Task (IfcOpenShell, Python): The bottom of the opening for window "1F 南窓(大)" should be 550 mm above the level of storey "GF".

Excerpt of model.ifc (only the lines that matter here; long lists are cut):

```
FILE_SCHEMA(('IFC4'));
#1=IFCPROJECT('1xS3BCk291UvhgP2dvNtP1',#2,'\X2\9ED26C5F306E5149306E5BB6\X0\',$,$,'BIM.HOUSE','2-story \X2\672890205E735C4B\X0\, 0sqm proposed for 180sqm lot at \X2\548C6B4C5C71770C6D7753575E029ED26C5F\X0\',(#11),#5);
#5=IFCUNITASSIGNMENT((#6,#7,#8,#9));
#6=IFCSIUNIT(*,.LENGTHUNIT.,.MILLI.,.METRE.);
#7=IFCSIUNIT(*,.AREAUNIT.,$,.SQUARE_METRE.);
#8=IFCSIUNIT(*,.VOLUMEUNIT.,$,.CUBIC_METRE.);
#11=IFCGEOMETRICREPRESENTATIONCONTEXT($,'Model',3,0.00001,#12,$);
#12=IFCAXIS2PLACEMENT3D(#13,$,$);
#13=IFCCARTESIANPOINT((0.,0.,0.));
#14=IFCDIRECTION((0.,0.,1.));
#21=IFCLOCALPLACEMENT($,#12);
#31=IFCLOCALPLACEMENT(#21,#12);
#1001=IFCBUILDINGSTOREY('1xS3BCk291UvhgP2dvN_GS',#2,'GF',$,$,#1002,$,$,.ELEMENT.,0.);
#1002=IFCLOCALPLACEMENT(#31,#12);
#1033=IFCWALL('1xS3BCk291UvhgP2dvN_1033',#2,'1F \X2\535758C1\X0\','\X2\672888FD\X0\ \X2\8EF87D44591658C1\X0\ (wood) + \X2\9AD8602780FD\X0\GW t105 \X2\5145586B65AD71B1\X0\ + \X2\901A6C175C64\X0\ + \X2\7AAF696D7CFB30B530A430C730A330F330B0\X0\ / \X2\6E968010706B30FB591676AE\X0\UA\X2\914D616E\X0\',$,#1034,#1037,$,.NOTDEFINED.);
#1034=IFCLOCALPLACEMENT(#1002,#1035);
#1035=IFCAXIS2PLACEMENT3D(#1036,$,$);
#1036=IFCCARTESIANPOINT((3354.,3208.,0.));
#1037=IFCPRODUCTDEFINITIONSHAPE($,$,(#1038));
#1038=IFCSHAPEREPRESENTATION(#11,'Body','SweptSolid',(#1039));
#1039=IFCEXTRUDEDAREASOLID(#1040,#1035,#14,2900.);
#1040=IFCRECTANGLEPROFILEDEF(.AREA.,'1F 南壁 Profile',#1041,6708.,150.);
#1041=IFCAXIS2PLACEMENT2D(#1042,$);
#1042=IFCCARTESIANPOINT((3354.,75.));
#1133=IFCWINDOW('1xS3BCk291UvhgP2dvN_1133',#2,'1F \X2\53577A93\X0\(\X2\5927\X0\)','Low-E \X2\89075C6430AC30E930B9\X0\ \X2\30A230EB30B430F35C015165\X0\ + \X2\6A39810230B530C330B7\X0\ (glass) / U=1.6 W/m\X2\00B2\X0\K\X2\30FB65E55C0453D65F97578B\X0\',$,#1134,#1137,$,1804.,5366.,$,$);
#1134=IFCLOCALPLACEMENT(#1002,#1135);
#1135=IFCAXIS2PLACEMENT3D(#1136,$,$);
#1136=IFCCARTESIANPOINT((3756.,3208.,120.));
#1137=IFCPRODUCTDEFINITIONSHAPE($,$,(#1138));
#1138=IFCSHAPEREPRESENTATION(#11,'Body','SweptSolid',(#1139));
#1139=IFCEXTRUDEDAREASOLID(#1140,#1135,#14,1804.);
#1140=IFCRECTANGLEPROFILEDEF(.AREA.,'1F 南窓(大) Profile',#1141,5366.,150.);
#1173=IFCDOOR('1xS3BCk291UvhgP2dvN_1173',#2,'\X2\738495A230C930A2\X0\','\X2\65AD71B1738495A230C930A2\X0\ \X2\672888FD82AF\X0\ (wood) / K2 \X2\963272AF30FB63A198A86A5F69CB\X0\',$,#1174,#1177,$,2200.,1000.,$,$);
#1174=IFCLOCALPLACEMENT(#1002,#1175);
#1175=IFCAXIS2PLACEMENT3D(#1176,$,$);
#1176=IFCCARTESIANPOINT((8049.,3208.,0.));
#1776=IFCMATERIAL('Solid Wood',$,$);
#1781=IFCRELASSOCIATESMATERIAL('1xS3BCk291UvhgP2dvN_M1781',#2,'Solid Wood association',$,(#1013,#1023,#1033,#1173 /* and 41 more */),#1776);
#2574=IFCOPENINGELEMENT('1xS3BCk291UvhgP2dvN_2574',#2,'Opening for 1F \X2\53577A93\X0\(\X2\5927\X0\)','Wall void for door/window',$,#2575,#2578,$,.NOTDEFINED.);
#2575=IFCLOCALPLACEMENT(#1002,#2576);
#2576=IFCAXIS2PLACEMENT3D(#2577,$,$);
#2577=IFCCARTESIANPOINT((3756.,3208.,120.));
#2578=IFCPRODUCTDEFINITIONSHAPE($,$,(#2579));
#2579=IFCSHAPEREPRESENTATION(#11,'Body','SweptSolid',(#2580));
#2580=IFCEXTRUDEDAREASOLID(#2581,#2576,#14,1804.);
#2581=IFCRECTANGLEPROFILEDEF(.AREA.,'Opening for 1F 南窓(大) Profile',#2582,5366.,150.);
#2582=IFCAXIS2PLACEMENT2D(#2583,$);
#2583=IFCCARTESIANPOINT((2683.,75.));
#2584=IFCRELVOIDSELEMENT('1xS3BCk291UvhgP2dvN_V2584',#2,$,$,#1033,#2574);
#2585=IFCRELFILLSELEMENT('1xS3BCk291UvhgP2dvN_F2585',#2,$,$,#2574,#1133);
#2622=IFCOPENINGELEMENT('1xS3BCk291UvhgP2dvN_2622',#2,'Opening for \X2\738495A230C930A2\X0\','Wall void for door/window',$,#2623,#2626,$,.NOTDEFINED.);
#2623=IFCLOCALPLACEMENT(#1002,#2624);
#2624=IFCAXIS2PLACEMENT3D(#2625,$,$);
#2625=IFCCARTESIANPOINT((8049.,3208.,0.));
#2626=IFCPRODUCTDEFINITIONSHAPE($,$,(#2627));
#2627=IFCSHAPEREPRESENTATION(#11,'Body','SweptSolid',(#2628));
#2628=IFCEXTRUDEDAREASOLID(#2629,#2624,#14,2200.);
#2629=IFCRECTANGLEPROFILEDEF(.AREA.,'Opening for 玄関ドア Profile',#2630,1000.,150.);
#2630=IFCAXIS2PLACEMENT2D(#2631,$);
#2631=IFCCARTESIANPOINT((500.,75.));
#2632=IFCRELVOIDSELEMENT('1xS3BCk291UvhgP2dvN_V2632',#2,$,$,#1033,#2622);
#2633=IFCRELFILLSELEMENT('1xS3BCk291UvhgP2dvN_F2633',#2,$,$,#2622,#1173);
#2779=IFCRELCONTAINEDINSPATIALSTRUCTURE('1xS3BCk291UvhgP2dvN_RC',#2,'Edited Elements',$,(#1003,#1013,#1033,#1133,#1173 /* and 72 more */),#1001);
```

```python
import numpy as np
import ifcopenshell
import ifcopenshell.api.geometry
import ifcopenshell.geom
import ifcopenshell.util.element
import ifcopenshell.util.placement
import ifcopenshell.util.shape
import ifcopenshell.util.unit

model = ifcopenshell.open("model.ifc")
unit_scale = ifcopenshell.util.unit.calculate_unit_scale(model)

window = model.by_guid("1xS3BCk291UvhgP2dvN_1133")
opening = window.FillsVoids[0].RelatingOpeningElement
storey = ifcopenshell.util.element.get_container(window, ifc_class="IfcBuildingStorey")
level = ifcopenshell.util.placement.get_local_placement(storey.ObjectPlacement)[2, 3]

# The opening's origin need not be at the sill, so measure its lowest point.
shape = ifcopenshell.geom.create_shape(ifcopenshell.geom.settings(), opening)
bottom = ifcopenshell.util.shape.get_shape_bottom_elevation(shape, shape.geometry) / unit_scale
dz = level + 0.55 / unit_scale - bottom

shift = np.array([0.0, 0.0, dz])
# The window is not placed relative to its opening, so move both.
for product in (opening, window):
    matrix = ifcopenshell.util.placement.get_local_placement(product.ObjectPlacement)
    matrix[:3, 3] += shift
    ifcopenshell.api.geometry.edit_object_placement(model, product=product, matrix=matrix, is_si=False)

print(f"moved by {dz * unit_scale:+.3f} m")

model.write("model_v2.ifc")
```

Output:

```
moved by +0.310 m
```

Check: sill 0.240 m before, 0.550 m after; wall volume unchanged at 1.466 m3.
